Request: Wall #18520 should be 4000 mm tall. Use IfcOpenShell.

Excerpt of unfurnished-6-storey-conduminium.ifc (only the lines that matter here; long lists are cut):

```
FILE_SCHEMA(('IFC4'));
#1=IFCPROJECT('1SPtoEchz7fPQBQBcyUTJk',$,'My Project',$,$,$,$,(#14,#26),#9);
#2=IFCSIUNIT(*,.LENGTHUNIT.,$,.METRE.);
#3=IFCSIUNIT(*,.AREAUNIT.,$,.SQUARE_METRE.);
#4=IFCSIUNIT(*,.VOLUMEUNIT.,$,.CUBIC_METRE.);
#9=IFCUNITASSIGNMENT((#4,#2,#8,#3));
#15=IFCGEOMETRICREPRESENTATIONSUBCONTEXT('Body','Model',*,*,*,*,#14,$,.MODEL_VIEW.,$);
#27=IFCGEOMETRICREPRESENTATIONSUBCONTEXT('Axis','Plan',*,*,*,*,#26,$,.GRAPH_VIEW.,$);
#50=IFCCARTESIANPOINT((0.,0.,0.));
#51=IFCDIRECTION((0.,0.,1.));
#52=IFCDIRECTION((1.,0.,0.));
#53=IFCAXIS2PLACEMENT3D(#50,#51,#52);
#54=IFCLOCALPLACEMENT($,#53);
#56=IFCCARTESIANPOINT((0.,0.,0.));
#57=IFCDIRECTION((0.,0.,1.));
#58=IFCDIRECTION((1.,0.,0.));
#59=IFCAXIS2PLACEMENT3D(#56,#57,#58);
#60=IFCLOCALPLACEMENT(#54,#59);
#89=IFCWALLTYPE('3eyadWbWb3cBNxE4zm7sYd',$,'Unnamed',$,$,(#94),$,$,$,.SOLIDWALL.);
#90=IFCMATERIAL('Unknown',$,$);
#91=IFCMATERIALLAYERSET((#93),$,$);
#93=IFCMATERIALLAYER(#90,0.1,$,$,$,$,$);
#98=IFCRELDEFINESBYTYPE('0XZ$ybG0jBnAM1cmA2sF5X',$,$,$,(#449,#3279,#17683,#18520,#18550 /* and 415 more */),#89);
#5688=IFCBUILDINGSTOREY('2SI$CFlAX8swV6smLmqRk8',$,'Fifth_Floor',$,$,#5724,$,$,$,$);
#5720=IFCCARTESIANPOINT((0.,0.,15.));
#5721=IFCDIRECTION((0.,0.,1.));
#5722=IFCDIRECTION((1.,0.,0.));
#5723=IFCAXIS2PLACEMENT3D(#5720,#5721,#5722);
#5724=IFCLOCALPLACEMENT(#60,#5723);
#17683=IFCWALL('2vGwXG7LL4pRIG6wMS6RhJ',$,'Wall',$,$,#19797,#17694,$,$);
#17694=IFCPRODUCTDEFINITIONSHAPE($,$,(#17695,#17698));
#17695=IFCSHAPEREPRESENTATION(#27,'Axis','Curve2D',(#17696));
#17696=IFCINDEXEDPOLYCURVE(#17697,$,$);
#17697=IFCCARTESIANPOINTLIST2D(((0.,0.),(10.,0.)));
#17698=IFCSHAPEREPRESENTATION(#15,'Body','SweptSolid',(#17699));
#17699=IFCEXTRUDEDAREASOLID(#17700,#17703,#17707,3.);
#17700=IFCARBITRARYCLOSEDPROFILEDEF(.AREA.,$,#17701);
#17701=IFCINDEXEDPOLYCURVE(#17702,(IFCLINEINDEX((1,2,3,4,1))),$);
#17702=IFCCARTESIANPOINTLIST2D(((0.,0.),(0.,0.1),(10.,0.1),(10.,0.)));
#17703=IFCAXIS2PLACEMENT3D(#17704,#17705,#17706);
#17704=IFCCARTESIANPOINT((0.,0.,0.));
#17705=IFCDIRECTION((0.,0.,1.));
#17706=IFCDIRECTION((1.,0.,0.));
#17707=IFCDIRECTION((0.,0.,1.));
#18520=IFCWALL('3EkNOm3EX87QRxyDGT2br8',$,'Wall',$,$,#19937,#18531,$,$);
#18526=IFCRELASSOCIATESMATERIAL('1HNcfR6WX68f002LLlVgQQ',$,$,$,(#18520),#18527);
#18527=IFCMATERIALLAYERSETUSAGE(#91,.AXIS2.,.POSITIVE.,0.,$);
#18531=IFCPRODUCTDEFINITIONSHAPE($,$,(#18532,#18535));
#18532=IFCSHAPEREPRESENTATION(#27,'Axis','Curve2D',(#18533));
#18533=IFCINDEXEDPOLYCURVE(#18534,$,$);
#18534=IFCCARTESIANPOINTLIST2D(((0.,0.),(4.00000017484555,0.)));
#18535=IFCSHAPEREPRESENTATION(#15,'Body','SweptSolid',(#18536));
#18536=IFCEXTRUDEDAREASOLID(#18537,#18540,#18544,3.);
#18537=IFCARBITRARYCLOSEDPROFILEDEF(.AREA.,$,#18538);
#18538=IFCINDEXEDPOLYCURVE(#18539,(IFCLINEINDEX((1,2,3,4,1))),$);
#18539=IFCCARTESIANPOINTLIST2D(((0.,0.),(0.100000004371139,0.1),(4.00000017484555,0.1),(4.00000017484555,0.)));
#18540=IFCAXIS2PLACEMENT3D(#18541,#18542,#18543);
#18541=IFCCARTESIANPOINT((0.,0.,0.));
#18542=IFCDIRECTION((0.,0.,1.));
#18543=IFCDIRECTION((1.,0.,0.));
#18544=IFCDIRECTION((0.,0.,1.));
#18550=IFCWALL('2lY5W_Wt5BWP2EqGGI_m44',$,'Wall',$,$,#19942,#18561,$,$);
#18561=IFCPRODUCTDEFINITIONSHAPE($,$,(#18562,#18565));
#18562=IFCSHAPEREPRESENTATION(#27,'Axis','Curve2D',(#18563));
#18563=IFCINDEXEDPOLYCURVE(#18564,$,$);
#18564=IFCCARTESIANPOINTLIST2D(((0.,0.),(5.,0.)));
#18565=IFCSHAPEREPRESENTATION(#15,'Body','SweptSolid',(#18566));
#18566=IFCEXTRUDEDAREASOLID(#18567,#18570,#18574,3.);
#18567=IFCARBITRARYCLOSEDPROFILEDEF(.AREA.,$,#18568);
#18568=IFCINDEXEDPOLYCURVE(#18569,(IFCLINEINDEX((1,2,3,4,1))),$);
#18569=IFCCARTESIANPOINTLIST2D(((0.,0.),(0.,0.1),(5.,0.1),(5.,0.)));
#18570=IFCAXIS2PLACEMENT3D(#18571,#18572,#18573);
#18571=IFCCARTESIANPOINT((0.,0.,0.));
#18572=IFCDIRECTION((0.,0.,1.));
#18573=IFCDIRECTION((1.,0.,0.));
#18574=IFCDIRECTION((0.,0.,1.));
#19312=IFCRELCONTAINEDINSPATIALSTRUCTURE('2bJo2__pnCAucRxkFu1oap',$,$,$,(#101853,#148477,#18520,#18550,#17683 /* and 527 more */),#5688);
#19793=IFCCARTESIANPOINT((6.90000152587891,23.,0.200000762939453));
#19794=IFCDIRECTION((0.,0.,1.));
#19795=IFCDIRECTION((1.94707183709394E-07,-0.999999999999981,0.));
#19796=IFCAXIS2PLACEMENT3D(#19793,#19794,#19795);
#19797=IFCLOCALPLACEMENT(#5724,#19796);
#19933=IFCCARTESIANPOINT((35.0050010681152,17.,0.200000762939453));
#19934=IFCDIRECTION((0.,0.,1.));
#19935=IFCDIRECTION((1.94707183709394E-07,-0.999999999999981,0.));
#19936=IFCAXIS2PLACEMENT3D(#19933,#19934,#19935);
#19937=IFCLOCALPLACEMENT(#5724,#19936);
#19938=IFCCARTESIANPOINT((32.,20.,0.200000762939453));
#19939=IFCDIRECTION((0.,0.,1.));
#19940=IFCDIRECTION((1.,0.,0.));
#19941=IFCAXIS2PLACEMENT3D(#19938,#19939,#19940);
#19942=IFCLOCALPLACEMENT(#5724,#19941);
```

```python
import ifcopenshell
import ifcopenshell.geom
import ifcopenshell.util.representation
import ifcopenshell.util.shape
import ifcopenshell.util.unit

model = ifcopenshell.open("unfurnished-6-storey-conduminium.ifc")
unit_scale = ifcopenshell.util.unit.calculate_unit_scale(model)
settings = ifcopenshell.geom.settings()


def volume(element):
    """Net volume in cubic metres, openings subtracted."""
    shape = ifcopenshell.geom.create_shape(settings, element)
    return ifcopenshell.util.shape.get_volume(shape.geometry)


wall = model.by_guid("3EkNOm3EX87QRxyDGT2br8")
before = volume(wall)

body = ifcopenshell.util.representation.get_representation(wall, "Model", "Body")
solid = body.Items[0]
old_height = solid.Depth
solid.Depth = 4 / unit_scale
after = volume(wall)

print(f"height {old_height:g} -> {solid.Depth:g}, volume {before:.3f} -> {after:.3f} m3")

model.write("unfurnished-6-storey-conduminium_updated.ifc")
```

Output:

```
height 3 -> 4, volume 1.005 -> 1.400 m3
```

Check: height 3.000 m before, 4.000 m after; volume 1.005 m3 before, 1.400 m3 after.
